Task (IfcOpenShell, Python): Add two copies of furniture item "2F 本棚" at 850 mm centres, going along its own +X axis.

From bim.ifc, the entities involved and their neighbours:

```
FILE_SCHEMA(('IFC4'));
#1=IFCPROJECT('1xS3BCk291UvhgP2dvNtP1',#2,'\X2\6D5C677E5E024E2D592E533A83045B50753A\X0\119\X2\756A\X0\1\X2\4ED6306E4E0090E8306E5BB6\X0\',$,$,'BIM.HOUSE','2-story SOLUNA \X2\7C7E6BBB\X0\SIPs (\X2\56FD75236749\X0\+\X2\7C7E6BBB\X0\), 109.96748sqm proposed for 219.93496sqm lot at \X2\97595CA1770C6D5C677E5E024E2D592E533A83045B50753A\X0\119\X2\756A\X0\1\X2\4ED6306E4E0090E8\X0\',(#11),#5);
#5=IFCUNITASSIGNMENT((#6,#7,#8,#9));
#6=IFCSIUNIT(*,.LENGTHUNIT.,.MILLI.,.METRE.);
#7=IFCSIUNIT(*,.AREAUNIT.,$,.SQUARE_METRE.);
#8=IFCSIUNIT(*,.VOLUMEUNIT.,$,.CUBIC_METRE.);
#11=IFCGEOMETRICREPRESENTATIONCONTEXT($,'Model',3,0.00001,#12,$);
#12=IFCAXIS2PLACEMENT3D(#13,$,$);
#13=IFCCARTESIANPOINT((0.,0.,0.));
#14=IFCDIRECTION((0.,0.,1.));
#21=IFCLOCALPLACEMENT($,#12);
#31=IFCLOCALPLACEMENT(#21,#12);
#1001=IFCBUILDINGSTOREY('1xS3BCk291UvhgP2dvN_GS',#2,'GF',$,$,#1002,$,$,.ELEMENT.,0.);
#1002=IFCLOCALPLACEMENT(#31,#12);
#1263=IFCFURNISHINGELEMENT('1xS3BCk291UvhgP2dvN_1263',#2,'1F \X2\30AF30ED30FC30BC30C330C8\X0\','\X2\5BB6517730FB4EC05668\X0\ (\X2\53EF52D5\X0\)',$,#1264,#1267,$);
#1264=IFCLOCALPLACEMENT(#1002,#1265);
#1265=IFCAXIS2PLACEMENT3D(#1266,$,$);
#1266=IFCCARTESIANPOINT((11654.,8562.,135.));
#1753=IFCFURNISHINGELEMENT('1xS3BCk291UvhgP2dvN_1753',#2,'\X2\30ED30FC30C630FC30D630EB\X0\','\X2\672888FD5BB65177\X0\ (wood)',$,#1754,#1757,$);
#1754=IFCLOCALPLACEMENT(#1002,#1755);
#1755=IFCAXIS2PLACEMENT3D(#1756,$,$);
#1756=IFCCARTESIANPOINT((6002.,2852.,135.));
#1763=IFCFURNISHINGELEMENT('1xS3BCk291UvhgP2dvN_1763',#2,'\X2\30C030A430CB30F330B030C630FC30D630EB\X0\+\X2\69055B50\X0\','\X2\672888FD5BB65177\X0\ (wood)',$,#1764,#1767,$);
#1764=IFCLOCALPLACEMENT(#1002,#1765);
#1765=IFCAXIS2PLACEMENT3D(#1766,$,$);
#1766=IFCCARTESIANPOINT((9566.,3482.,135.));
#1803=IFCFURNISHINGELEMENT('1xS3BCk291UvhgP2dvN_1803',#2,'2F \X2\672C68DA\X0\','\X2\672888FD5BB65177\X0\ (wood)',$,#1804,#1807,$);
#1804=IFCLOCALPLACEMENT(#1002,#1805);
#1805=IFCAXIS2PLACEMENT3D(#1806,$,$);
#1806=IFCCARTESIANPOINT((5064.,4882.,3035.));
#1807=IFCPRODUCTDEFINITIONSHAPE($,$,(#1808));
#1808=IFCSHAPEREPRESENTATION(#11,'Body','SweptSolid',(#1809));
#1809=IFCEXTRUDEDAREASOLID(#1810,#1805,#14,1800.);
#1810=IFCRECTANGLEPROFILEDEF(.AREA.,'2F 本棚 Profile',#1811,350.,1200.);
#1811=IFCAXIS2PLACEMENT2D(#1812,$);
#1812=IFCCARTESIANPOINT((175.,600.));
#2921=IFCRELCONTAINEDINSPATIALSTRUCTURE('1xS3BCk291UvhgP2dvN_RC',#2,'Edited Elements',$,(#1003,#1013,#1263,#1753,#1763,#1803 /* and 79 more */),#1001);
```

```python
import ifcopenshell
import ifcopenshell.api.geometry
import ifcopenshell.api.root
import ifcopenshell.util.element
import ifcopenshell.util.placement

model = ifcopenshell.open("bim.ifc")


def reuse_history(source, copy):
    """copy_class also copies each property set's owner history, people and application; keep the originals."""
    for rel in copy.IsDefinedBy:
        if rel.is_a("IfcRelDefinesByProperties") and (history := rel.RelatingPropertyDefinition.OwnerHistory):
            rel.RelatingPropertyDefinition.OwnerHistory = source.OwnerHistory
            ifcopenshell.util.element.remove_deep2(model, history)


source = model.by_guid("1xS3BCk291UvhgP2dvN_1803")
base = ifcopenshell.util.placement.get_local_placement(source.ObjectPlacement)
step = base[:3, 0] * 850.0

for i in range(1, 3):
    copy = ifcopenshell.api.root.copy_class(model, product=source)
    copy.Representation = ifcopenshell.util.element.copy_deep(
        model, source.Representation, exclude=["IfcGeometricRepresentationContext", "IfcRepresentationMap"]
    )
    reuse_history(source, copy)
    matrix = base.copy()
    matrix[:3, 3] += i * step
    print("added at", matrix[:3, 3].round(3) + 0.0)
    ifcopenshell.api.geometry.edit_object_placement(model, product=copy, matrix=matrix, is_si=False)

model.write("bim_updated.ifc")
```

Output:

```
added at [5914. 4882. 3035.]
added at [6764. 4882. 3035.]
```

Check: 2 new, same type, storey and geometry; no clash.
